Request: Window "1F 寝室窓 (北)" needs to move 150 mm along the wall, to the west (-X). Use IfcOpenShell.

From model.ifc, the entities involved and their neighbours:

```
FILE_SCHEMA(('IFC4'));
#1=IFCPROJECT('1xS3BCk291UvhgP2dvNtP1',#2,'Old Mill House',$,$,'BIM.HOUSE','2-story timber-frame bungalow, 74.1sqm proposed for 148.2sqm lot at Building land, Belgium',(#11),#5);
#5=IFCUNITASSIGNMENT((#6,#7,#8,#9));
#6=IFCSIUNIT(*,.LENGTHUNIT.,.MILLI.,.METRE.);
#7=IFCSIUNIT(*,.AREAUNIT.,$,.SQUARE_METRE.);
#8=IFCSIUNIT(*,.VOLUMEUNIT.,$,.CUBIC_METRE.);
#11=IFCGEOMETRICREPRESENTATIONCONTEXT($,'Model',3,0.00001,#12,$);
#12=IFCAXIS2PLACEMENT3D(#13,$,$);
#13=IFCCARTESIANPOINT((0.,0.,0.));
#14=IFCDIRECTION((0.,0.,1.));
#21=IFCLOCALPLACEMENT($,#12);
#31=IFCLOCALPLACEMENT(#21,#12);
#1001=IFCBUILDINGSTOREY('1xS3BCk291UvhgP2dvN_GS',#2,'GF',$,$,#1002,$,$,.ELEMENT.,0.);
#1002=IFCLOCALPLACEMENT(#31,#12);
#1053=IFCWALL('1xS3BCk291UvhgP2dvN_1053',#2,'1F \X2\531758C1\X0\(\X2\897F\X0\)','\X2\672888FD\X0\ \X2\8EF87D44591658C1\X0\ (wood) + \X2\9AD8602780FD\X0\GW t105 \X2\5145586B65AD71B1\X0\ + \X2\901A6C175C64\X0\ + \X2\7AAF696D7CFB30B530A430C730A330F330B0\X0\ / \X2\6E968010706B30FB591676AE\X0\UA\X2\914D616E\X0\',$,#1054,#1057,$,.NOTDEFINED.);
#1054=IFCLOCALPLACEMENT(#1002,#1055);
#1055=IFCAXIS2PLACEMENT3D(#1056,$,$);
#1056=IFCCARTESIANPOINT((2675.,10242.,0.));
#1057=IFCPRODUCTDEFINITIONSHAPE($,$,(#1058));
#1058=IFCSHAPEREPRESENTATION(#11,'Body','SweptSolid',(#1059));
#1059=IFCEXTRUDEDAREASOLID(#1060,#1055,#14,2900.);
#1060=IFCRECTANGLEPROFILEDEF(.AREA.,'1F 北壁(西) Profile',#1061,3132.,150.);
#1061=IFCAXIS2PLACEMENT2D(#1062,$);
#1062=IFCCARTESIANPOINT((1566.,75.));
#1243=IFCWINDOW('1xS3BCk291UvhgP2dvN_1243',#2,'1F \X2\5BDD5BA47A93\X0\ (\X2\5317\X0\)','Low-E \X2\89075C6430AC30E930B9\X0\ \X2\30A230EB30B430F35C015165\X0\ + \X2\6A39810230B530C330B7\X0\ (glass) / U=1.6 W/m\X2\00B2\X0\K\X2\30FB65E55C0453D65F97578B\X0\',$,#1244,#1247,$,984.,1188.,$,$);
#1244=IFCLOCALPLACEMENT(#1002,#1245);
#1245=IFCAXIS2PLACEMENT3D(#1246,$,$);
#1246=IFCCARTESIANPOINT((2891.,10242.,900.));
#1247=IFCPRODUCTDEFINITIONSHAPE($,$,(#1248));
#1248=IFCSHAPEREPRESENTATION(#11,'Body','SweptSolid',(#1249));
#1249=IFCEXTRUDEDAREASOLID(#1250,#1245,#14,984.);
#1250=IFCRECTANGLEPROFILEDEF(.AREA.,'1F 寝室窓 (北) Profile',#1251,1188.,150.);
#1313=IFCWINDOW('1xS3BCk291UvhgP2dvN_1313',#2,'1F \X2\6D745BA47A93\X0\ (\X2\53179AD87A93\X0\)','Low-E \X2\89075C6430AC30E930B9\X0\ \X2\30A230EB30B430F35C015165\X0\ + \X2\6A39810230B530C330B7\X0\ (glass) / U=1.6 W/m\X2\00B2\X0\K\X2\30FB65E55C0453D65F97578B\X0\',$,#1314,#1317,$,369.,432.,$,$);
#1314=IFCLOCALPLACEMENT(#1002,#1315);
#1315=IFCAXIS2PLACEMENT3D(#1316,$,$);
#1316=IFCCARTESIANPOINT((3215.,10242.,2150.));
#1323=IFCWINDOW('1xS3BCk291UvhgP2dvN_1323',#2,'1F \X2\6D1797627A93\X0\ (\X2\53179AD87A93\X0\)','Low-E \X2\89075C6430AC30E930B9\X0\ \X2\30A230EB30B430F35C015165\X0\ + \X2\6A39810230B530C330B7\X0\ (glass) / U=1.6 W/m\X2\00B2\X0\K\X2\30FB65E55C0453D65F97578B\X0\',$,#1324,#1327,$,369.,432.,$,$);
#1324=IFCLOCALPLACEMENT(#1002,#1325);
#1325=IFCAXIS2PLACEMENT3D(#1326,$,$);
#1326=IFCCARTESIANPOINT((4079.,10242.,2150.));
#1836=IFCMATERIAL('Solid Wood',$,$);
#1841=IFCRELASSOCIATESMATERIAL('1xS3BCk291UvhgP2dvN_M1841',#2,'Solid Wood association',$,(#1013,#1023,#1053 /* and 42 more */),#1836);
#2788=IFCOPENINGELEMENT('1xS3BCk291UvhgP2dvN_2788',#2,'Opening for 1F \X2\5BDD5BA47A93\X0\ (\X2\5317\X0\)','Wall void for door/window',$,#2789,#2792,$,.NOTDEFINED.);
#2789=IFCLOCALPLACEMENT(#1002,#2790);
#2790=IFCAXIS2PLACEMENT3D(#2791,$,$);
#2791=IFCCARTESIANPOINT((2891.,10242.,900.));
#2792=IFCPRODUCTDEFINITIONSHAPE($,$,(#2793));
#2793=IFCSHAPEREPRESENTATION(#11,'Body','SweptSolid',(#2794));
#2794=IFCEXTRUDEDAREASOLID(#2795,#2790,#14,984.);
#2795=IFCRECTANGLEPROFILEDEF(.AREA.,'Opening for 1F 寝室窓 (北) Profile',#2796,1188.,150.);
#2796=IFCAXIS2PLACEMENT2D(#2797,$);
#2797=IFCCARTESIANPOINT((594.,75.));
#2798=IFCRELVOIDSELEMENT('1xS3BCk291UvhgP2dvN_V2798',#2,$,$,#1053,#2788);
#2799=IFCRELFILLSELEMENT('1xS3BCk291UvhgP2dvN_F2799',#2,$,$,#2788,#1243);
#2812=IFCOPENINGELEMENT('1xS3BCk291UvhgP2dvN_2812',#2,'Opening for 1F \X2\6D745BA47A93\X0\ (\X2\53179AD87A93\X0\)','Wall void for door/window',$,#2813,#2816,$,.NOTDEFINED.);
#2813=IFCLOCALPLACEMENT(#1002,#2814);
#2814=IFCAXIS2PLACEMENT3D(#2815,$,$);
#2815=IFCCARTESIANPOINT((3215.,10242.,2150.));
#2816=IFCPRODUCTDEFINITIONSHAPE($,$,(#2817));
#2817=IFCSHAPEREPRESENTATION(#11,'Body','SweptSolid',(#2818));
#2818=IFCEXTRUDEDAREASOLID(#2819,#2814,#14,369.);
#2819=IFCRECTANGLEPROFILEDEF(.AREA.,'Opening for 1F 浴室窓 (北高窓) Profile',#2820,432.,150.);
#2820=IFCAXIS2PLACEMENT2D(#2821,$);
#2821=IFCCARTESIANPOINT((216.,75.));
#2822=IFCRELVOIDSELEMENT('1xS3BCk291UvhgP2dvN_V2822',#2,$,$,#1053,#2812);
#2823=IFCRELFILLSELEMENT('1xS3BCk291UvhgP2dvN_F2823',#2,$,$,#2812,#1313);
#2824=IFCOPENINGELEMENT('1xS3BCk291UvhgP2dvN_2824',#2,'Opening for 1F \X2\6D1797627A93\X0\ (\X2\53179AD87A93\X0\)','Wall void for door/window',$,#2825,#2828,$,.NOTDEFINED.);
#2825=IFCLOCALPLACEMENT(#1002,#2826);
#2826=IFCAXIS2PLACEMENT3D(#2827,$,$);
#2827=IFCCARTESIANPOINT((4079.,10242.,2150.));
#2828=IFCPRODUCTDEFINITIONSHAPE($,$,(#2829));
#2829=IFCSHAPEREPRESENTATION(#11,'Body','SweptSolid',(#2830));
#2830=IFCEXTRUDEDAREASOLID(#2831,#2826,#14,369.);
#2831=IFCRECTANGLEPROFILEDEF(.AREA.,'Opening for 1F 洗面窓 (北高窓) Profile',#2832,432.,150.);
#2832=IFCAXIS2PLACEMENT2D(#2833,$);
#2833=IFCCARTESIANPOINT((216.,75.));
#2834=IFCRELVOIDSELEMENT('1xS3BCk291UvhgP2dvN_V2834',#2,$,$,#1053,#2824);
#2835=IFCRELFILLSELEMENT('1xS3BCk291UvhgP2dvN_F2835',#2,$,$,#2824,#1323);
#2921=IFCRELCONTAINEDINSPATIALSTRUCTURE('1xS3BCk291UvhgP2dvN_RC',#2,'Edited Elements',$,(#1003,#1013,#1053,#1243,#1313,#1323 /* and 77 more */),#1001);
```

```python
import ifcopenshell
import ifcopenshell.api.geometry
import ifcopenshell.util.placement
import ifcopenshell.util.unit

model = ifcopenshell.open("model.ifc")
unit_scale = ifcopenshell.util.unit.calculate_unit_scale(model)

window = model.by_guid("1xS3BCk291UvhgP2dvN_1243")
opening = window.FillsVoids[0].RelatingOpeningElement
wall = opening.VoidsElements[0].RelatingBuildingElement

wall_matrix = ifcopenshell.util.placement.get_local_placement(wall.ObjectPlacement)
shift = wall_matrix[:3, 0] * -0.15 / unit_scale
before = ifcopenshell.util.placement.get_local_placement(window.ObjectPlacement)[:3, 3].copy()

# The window is not placed relative to its opening, so move both.
for product in (opening, window):
    matrix = ifcopenshell.util.placement.get_local_placement(product.ObjectPlacement)
    matrix[:3, 3] += shift
    ifcopenshell.api.geometry.edit_object_placement(model, product=product, matrix=matrix, is_si=False)

after = ifcopenshell.util.placement.get_local_placement(window.ObjectPlacement)[:3, 3]
print("window moved by", (after - before).round(3) + 0.0)

model.write("model-out.ifc")
```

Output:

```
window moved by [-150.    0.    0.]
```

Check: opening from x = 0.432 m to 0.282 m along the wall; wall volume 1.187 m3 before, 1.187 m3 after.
